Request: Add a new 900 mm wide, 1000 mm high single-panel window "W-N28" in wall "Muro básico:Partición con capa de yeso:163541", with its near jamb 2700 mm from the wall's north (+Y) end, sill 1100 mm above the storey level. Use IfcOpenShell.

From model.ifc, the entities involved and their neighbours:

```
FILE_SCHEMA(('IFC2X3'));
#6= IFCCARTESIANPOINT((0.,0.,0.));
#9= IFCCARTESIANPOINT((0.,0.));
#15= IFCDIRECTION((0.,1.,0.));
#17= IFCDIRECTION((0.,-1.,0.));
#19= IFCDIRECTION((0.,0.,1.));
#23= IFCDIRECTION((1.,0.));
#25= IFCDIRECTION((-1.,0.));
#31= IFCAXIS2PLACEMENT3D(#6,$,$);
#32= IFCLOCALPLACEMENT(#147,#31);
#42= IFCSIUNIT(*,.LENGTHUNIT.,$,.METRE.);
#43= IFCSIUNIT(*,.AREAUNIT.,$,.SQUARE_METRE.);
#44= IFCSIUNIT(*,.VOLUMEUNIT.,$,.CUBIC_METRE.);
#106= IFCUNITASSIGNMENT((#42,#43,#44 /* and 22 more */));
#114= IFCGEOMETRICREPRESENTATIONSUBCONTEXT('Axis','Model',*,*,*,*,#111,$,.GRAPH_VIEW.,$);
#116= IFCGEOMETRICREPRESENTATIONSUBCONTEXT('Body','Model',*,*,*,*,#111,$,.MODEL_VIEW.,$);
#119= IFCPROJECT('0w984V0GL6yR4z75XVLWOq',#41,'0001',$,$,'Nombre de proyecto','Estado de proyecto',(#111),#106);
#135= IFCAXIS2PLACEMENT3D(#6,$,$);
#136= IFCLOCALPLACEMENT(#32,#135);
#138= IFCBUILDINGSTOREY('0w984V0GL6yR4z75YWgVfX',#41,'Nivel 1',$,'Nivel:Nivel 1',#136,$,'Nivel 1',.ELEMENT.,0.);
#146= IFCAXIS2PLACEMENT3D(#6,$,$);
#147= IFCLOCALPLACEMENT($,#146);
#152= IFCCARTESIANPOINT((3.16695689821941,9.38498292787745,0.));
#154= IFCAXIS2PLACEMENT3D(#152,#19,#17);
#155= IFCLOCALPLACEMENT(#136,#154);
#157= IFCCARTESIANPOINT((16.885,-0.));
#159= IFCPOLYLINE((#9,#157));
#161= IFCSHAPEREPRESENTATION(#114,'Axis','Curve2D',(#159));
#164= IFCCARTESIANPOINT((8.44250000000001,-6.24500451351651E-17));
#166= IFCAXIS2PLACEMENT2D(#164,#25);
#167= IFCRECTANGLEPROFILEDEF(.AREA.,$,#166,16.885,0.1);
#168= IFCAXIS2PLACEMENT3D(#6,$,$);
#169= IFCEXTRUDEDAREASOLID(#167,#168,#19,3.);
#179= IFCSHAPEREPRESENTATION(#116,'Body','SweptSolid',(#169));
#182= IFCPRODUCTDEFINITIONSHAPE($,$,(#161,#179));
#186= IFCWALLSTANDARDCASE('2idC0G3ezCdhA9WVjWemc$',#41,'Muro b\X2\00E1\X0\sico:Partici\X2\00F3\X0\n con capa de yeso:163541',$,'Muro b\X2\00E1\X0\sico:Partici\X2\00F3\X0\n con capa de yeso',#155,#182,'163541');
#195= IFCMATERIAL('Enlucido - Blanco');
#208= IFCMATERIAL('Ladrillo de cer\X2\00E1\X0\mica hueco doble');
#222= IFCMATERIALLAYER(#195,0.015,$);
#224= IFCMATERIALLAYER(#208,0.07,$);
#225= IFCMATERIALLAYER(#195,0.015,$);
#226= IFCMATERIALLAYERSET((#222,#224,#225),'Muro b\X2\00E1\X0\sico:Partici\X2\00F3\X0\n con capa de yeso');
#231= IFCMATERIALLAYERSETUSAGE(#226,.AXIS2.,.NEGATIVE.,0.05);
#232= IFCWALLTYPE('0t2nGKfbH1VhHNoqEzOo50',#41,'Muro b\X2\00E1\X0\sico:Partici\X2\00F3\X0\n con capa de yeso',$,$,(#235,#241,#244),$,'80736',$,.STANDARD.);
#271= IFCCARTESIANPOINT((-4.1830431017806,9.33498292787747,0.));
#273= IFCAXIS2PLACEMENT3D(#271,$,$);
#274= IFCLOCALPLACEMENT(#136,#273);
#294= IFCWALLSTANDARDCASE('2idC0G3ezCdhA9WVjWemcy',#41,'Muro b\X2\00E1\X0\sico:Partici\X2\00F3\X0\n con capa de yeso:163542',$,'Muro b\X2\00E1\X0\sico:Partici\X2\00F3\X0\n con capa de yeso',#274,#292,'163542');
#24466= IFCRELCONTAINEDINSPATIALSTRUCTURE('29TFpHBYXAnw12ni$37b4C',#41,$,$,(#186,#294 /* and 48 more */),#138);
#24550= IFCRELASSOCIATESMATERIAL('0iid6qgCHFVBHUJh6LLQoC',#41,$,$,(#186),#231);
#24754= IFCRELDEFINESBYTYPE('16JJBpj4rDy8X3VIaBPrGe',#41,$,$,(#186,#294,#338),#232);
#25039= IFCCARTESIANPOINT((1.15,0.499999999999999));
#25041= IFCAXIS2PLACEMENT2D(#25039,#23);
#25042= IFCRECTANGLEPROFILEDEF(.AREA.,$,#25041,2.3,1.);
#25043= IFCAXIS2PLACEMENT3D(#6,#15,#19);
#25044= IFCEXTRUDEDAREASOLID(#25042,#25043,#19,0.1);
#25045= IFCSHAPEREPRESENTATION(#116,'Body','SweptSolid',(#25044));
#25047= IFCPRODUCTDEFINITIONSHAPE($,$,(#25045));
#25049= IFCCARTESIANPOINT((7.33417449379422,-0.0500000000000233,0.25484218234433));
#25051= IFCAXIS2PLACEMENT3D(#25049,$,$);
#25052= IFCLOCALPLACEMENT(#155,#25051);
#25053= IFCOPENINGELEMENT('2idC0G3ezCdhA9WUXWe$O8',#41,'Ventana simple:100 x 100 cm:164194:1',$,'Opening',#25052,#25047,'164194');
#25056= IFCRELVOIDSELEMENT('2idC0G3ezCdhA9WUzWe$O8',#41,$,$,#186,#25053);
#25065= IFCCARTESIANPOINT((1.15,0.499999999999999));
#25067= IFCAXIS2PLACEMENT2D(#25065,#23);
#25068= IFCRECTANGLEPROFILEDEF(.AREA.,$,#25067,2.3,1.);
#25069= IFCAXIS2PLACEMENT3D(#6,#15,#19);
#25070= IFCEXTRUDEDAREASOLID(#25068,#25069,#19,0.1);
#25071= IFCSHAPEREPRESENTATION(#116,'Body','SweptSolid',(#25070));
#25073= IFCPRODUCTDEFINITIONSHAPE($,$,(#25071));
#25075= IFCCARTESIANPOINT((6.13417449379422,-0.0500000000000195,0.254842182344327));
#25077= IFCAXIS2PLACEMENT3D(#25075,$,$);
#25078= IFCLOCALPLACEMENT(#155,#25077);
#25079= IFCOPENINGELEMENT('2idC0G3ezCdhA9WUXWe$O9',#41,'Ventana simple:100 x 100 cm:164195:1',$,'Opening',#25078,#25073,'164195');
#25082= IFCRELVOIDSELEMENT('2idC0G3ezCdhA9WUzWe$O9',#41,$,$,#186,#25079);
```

```python
import numpy as np
import ifcopenshell
import ifcopenshell.api.feature
import ifcopenshell.api.geometry
import ifcopenshell.api.root
import ifcopenshell.api.spatial
import ifcopenshell.api.type
import ifcopenshell.geom
import ifcopenshell.util.element
import ifcopenshell.util.placement
import ifcopenshell.util.representation
import ifcopenshell.util.shape
import ifcopenshell.util.unit

model = ifcopenshell.open("model.ifc")
unit_scale = ifcopenshell.util.unit.calculate_unit_scale(model)
settings = ifcopenshell.geom.settings()


def volume(element):
    """Net volume in cubic metres, openings subtracted."""
    shape = ifcopenshell.geom.create_shape(settings, element)
    return ifcopenshell.util.shape.get_volume(shape.geometry)


wall = model.by_guid("2idC0G3ezCdhA9WVjWemc$")
storey = ifcopenshell.util.element.get_container(wall, ifc_class="IfcBuildingStorey")
context = ifcopenshell.util.representation.get_context(model, "Model", "Body", "MODEL_VIEW")
before = volume(wall)

width, height, from_end, sill = 0.9, 1, 2.7, 1.1  # metres

# The wall runs along its own X axis, and the end named is its -X end.
wall_shape = ifcopenshell.geom.create_shape(settings, wall)
x, y, z = ifcopenshell.util.shape.get_vertices(wall_shape.geometry).T
start = x.min() + from_end
face, thickness = float(y.min()), float(y.max() - y.min())
wall_matrix = ifcopenshell.util.placement.get_local_placement(wall.ObjectPlacement)
level = ifcopenshell.util.placement.get_local_placement(storey.ObjectPlacement)[2, 3]


def in_wall(x, y):
    """Placement at x, y metres in the wall's axes, at sill height."""
    matrix = wall_matrix.copy()
    matrix[:, 3] = wall_matrix @ np.array([x / unit_scale, y / unit_scale, 0.0, 1.0])
    matrix[2, 3] = level + sill / unit_scale
    return matrix


# Opening: a box that overshoots both wall faces by 50 mm.
opening = ifcopenshell.api.root.create_entity(model, ifc_class="IfcOpeningElement")
box = ifcopenshell.api.geometry.add_wall_representation(
    model, context=context, length=width, height=height, thickness=thickness + 0.1
)
ifcopenshell.api.geometry.assign_representation(model, product=opening, representation=box)
ifcopenshell.api.geometry.edit_object_placement(model, product=opening, matrix=in_wall(start, face - 0.05), is_si=False)
ifcopenshell.api.feature.add_feature(model, feature=opening, element=wall)

window = ifcopenshell.api.root.create_entity(model, ifc_class="IfcWindow", name="W-N28")
window.OverallWidth, window.OverallHeight = width / unit_scale, height / unit_scale
body = ifcopenshell.api.geometry.add_window_representation(
    model,
    context=context,
    overall_width=window.OverallWidth,
    overall_height=window.OverallHeight,
    partition_type="SINGLE_PANEL",
)
ifcopenshell.api.geometry.assign_representation(model, product=window, representation=body)
ifcopenshell.api.spatial.assign_container(model, products=[window], relating_structure=storey)
fills = ifcopenshell.api.feature.add_filling(model, opening=opening, element=window)
fills.OwnerHistory = window.OwnerHistory  # required in IFC2X3

# IFC2X3 keeps the operation on the window style.
style = ifcopenshell.api.root.create_entity(model, ifc_class="IfcWindowStyle", name="W-N28")
style.OperationType, style.ConstructionType = "SINGLE_PANEL", "NOTDEFINED"
style.ParameterTakesPrecedence = style.Sizeable = False
ifcopenshell.api.type.assign_type(model, related_objects=[window], relating_type=style)

# Centre the window in the wall's thickness.
ifcopenshell.api.geometry.edit_object_placement(model, product=window, matrix=in_wall(start, face), is_si=False)
window_shape = ifcopenshell.geom.create_shape(settings, window)
depth = ifcopenshell.util.shape.get_vertices(window_shape.geometry)[:, 1]
offset = face + thickness / 2 - (depth.min() + depth.max()) / 2
ifcopenshell.api.geometry.edit_object_placement(model, product=window, matrix=in_wall(start, offset), is_si=False)

after = volume(wall)

print(f"wall volume {before:.3f} -> {after:.3f} m3")

model.write("model-out.ifc")
```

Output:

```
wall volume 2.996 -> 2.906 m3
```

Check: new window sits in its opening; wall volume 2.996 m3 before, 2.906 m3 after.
